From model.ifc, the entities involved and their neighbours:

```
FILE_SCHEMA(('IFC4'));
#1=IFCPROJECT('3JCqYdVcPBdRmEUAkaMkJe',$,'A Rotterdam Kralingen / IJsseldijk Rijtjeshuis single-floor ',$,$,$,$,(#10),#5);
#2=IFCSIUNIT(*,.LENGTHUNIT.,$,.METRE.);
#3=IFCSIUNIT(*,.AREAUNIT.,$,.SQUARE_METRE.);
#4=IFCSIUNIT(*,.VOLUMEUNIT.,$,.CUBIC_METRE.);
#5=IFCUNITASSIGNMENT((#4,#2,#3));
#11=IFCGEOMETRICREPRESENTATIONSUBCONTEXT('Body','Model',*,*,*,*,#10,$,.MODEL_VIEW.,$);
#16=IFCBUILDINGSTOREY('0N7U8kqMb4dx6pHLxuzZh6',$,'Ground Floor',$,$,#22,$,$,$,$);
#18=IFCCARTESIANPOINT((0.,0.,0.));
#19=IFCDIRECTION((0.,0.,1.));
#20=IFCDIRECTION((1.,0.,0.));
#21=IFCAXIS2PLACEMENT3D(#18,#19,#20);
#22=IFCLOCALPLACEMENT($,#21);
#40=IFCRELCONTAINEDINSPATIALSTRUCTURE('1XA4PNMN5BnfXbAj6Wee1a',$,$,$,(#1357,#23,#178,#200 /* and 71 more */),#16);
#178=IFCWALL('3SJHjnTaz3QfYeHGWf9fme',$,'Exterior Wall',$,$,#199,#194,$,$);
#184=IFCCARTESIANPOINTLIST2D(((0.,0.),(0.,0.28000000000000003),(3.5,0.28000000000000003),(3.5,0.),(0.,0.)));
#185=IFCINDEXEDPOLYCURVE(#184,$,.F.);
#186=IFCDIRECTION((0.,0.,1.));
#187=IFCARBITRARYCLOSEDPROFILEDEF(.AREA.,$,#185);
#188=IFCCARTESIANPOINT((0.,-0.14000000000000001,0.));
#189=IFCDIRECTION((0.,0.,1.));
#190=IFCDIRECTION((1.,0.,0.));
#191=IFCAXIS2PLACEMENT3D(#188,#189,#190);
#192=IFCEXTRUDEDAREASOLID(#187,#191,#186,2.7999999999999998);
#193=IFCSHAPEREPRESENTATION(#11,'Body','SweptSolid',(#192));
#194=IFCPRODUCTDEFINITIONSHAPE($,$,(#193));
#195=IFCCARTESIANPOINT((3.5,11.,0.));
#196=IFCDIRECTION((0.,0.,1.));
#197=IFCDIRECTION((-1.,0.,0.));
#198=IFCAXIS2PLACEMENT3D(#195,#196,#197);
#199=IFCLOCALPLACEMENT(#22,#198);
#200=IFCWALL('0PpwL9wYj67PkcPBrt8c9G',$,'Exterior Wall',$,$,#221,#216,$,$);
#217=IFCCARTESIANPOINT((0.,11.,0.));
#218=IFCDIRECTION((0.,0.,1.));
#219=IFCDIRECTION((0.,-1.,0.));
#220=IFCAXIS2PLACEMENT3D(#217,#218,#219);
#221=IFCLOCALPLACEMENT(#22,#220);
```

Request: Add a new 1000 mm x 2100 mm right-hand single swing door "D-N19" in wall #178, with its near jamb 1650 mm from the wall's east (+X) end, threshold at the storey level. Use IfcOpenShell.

```python
import numpy as np
import ifcopenshell
import ifcopenshell.api.feature
import ifcopenshell.api.geometry
import ifcopenshell.api.root
import ifcopenshell.api.spatial
import ifcopenshell.geom
import ifcopenshell.util.element
import ifcopenshell.util.placement
import ifcopenshell.util.representation
import ifcopenshell.util.shape
import ifcopenshell.util.unit

model = ifcopenshell.open("model.ifc")
unit_scale = ifcopenshell.util.unit.calculate_unit_scale(model)
settings = ifcopenshell.geom.settings()


def volume(element):
    """Net volume in cubic metres, openings subtracted."""
    shape = ifcopenshell.geom.create_shape(settings, element)
    return ifcopenshell.util.shape.get_volume(shape.geometry)


wall = model.by_guid("3SJHjnTaz3QfYeHGWf9fme")
storey = ifcopenshell.util.element.get_container(wall, ifc_class="IfcBuildingStorey")
context = ifcopenshell.util.representation.get_context(model, "Model", "Body", "MODEL_VIEW")
before = volume(wall)

width, height, from_end, sill = 1, 2.1, 1.65, 0.0  # metres

# The wall runs along its own X axis, and the end named is its -X end.
wall_shape = ifcopenshell.geom.create_shape(settings, wall)
x, y, z = ifcopenshell.util.shape.get_vertices(wall_shape.geometry).T
start = x.min() + from_end
face, thickness = float(y.min()), float(y.max() - y.min())
wall_matrix = ifcopenshell.util.placement.get_local_placement(wall.ObjectPlacement)
level = ifcopenshell.util.placement.get_local_placement(storey.ObjectPlacement)[2, 3]


def in_wall(x, y):
    """Placement at x, y metres in the wall's axes, at sill height."""
    matrix = wall_matrix.copy()
    matrix[:, 3] = wall_matrix @ np.array([x / unit_scale, y / unit_scale, 0.0, 1.0])
    matrix[2, 3] = level + sill / unit_scale
    return matrix


# Opening: a box that overshoots both wall faces by 50 mm.
opening = ifcopenshell.api.root.create_entity(model, ifc_class="IfcOpeningElement", predefined_type="OPENING")
box = ifcopenshell.api.geometry.add_wall_representation(
    model, context=context, length=width, height=height, thickness=thickness + 0.1
)
ifcopenshell.api.geometry.assign_representation(model, product=opening, representation=box)
ifcopenshell.api.geometry.edit_object_placement(model, product=opening, matrix=in_wall(start, face - 0.05), is_si=False)
ifcopenshell.api.feature.add_feature(model, feature=opening, element=wall)

door = ifcopenshell.api.root.create_entity(model, ifc_class="IfcDoor", name="D-N19", predefined_type="DOOR")
door.OverallWidth, door.OverallHeight = width / unit_scale, height / unit_scale
door.OperationType = "SINGLE_SWING_RIGHT"
body = ifcopenshell.api.geometry.add_door_representation(
    model,
    context=context,
    overall_width=door.OverallWidth,
    overall_height=door.OverallHeight,
    operation_type="SINGLE_SWING_RIGHT",
    lining_properties={"LiningDepth": thickness / unit_scale, "ThresholdDepth": thickness / unit_scale},
)
ifcopenshell.api.geometry.assign_representation(model, product=door, representation=body)
ifcopenshell.api.spatial.assign_container(model, products=[door], relating_structure=storey)
ifcopenshell.api.feature.add_filling(model, opening=opening, element=door)

# The lining spans the wall, so the door starts at the wall face.
ifcopenshell.api.geometry.edit_object_placement(model, product=door, matrix=in_wall(start, face), is_si=False)

after = volume(wall)

print(f"wall volume {before:.3f} -> {after:.3f} m3")

model.write("model_rev.ifc")
```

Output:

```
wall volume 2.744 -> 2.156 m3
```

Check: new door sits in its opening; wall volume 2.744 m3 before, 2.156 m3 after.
